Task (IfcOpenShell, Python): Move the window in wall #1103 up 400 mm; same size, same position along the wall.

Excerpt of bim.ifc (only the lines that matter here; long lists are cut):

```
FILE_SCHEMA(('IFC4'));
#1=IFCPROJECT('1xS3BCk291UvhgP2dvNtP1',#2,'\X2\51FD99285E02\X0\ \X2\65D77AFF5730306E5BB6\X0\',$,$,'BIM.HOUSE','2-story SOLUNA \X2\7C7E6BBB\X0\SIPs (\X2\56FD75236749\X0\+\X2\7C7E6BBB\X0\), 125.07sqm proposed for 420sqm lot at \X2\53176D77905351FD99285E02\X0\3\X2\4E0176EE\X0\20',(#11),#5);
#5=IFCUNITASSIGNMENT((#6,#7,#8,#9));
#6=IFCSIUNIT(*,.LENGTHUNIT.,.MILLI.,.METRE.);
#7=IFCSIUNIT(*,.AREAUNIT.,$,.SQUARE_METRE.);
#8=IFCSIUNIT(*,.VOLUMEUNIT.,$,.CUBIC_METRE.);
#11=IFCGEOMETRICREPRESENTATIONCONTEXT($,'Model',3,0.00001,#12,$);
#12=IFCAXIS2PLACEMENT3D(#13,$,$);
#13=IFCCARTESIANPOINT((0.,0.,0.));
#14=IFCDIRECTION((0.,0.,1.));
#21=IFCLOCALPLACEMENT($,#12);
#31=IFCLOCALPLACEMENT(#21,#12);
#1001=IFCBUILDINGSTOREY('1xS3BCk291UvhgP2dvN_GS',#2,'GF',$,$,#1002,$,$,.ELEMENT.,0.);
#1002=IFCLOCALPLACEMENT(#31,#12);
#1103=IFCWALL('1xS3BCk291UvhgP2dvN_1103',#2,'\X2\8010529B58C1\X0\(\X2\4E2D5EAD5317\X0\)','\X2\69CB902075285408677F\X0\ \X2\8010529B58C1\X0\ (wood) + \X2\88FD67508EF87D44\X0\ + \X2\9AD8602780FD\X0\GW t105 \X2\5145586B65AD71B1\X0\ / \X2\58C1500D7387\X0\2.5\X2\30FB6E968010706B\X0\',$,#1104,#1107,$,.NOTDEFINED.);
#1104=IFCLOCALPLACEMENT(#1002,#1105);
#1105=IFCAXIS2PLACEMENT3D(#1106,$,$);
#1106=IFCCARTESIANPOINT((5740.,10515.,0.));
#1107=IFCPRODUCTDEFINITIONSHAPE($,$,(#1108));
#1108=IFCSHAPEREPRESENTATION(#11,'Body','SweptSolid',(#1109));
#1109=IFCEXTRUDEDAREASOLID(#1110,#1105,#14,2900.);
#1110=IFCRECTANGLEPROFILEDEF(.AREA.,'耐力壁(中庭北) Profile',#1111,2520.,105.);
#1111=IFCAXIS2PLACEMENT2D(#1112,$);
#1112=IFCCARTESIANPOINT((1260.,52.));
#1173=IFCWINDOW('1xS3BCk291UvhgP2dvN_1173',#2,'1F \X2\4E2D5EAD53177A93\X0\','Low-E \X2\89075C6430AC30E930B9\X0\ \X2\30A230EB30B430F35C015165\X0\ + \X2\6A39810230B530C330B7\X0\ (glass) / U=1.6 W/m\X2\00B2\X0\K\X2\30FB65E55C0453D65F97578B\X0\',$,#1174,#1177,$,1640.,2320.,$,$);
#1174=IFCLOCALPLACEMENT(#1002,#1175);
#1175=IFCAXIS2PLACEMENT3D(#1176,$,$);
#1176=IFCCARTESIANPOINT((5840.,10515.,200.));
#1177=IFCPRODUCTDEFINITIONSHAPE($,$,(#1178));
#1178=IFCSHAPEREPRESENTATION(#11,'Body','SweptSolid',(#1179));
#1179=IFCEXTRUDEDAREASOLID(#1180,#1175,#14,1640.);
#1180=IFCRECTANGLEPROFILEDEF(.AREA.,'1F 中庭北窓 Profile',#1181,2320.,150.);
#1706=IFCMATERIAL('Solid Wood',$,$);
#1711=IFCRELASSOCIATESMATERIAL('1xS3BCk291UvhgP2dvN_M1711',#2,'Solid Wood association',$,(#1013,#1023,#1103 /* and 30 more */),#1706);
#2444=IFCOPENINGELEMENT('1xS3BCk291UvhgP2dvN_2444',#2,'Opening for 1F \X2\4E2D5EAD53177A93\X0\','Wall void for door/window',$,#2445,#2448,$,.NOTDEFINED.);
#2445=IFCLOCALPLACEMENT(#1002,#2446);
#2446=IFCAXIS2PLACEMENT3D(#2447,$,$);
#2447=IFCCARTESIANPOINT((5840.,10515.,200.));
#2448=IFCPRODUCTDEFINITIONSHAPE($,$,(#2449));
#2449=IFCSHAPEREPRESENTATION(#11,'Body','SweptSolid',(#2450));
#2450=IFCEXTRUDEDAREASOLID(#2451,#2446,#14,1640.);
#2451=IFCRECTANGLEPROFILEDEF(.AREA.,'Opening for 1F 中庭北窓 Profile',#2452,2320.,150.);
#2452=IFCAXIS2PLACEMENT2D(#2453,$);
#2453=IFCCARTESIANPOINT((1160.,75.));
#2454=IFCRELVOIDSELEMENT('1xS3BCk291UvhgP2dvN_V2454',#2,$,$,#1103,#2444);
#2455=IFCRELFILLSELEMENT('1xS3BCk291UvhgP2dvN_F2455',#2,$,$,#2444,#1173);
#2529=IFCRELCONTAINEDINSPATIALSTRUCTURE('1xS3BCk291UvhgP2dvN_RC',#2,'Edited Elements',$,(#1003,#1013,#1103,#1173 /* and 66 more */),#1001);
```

```python
import numpy as np
import ifcopenshell
import ifcopenshell.api.geometry
import ifcopenshell.util.placement
import ifcopenshell.util.unit

model = ifcopenshell.open("bim.ifc")
unit_scale = ifcopenshell.util.unit.calculate_unit_scale(model)

window = model.by_guid("1xS3BCk291UvhgP2dvN_1173")
opening = window.FillsVoids[0].RelatingOpeningElement
dz = 400.0

shift = np.array([0.0, 0.0, dz])
# The window is not placed relative to its opening, so move both.
for product in (opening, window):
    matrix = ifcopenshell.util.placement.get_local_placement(product.ObjectPlacement)
    matrix[:3, 3] += shift
    ifcopenshell.api.geometry.edit_object_placement(model, product=product, matrix=matrix, is_si=False)

print(f"moved by {dz * unit_scale:+.3f} m")

model.write("bim_updated.ifc")
```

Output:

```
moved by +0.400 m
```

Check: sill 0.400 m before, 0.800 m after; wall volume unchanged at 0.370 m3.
